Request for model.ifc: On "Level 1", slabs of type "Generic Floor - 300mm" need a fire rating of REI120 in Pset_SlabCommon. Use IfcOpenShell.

First a look at what the model holds.

```python
import ifcopenshell
import ifcopenshell.util.element

model = ifcopenshell.open("model.ifc")
print(model.schema)
storey = next(s for s in model.by_type("IfcBuildingStorey") if s.Name == "Level 1")
slabs = [e for e in ifcopenshell.util.element.get_decomposition(storey) if e.is_a("IfcSlab")]
seen = {}
for e in slabs:
    element_type = ifcopenshell.util.element.get_type(e)
    key = (element_type.Name if element_type != e and element_type else None, ifcopenshell.util.element.get_pset(e, "Pset_SlabCommon", "FireRating"))
    seen[key] = seen.get(key, 0) + 1
for (name, value), count in sorted(seen.items(), key=str):
    print(count, "x", name, "|", value)
```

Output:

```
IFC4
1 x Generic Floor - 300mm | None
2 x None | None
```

```python
import ifcopenshell
import ifcopenshell.api.pset
import ifcopenshell.util.element

model = ifcopenshell.open("model.ifc")

storey = next(s for s in model.by_type("IfcBuildingStorey") if s.Name == "Level 1")
slabs = [e for e in ifcopenshell.util.element.get_decomposition(storey) if e.is_a("IfcSlab")]

count = 0
for e in slabs:
    element_type = ifcopenshell.util.element.get_type(e)
    if element_type in (None, e) or element_type.Name != "Generic Floor - 300mm":
        continue
    # add_pset returns the element's existing set when there is one.
    pset = ifcopenshell.api.pset.add_pset(model, product=e, name="Pset_SlabCommon")
    ifcopenshell.api.pset.edit_pset(model, pset=pset, properties={"FireRating": "REI120"})
    count += 1

print(count, "slabs updated")

model.write("model_rev.ifc")
```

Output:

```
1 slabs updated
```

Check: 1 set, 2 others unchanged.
